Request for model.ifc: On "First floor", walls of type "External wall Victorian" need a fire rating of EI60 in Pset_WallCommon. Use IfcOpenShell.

First a look at what the model holds.

```python
import ifcopenshell
import ifcopenshell.util.element

model = ifcopenshell.open("model.ifc")
print(model.schema)
storey = next(s for s in model.by_type("IfcBuildingStorey") if s.Name == "First floor")
walls = [e for e in ifcopenshell.util.element.get_decomposition(storey) if e.is_a("IfcWall")]
seen = {}
for e in walls:
    element_type = ifcopenshell.util.element.get_type(e)
    key = (element_type.Name if element_type != e and element_type else None, ifcopenshell.util.element.get_pset(e, "Pset_WallCommon", "FireRating"))
    seen[key] = seen.get(key, 0) + 1
for (name, value), count in sorted(seen.items(), key=str):
    print(count, "x", name, "|", value)
```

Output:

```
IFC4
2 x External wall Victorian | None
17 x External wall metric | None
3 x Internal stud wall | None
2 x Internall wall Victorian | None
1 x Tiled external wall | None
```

```python
import ifcopenshell
import ifcopenshell.api.pset
import ifcopenshell.util.element

model = ifcopenshell.open("model.ifc")

storey = next(s for s in model.by_type("IfcBuildingStorey") if s.Name == "First floor")
walls = [e for e in ifcopenshell.util.element.get_decomposition(storey) if e.is_a("IfcWall")]

count = 0
for e in walls:
    element_type = ifcopenshell.util.element.get_type(e)
    if element_type in (None, e) or element_type.Name != "External wall Victorian":
        continue
    # add_pset returns the element's existing set when there is one.
    pset = ifcopenshell.api.pset.add_pset(model, product=e, name="Pset_WallCommon")
    ifcopenshell.api.pset.edit_pset(model, pset=pset, properties={"FireRating": "EI60"})
    count += 1

print(count, "walls updated")

model.write("model_rev.ifc")
```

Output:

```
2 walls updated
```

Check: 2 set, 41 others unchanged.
